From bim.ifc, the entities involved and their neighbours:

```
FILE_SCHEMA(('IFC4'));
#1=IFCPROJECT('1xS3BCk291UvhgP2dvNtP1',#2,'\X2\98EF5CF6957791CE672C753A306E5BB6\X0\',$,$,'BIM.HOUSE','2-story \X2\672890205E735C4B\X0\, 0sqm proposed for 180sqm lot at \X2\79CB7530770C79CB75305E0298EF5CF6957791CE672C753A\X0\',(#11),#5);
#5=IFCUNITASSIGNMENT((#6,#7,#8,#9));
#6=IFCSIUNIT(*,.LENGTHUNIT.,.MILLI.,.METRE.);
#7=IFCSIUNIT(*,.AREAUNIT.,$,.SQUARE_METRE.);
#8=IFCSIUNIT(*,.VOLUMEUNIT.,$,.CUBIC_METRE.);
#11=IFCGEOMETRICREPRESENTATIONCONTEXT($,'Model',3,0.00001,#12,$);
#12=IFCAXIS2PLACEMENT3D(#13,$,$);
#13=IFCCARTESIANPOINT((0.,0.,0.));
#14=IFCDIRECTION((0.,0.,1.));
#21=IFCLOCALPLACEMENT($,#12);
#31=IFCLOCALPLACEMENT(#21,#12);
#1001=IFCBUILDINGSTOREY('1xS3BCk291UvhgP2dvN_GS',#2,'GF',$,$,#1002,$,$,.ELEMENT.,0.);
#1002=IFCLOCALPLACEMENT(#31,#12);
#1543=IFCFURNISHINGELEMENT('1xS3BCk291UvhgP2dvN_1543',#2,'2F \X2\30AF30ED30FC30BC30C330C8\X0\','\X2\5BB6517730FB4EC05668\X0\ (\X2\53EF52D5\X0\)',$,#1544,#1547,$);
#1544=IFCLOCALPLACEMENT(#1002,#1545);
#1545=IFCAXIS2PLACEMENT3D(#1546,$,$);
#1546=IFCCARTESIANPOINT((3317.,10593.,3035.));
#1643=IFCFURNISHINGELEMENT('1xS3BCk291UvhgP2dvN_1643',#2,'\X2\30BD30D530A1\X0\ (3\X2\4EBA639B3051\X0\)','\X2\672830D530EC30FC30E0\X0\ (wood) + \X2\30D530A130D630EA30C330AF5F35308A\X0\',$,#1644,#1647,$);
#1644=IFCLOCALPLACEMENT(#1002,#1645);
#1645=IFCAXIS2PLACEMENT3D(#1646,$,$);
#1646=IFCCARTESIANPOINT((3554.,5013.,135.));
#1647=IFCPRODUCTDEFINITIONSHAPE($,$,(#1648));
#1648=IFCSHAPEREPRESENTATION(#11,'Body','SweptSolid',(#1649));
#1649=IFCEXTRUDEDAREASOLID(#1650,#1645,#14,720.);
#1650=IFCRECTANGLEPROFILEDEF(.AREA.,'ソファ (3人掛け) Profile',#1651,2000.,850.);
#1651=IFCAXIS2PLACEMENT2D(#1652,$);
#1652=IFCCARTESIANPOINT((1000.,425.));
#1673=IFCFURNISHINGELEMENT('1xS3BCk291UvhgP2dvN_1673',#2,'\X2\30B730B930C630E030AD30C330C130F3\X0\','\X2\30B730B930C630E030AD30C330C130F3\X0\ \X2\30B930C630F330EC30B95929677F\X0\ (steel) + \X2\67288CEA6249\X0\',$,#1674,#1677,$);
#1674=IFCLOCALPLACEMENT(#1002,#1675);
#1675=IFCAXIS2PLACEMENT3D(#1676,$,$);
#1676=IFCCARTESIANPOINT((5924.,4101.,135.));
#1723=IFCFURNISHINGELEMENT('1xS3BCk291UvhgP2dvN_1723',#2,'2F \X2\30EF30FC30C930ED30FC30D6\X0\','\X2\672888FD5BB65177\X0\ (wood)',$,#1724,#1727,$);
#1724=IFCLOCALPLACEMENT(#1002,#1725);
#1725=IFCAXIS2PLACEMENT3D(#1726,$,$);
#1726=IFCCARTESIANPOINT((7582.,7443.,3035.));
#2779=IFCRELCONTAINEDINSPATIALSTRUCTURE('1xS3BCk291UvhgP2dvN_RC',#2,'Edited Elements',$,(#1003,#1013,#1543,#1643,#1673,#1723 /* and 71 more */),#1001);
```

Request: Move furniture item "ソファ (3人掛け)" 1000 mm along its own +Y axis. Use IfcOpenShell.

```python
import ifcopenshell
import ifcopenshell.api.geometry
import ifcopenshell.util.placement
import ifcopenshell.util.unit

model = ifcopenshell.open("bim.ifc")
unit_scale = ifcopenshell.util.unit.calculate_unit_scale(model)

item = model.by_id(1643)
matrix = ifcopenshell.util.placement.get_local_placement(item.ObjectPlacement)
matrix[:3, 3] += matrix[:3, 1] * 1 / unit_scale
ifcopenshell.api.geometry.edit_object_placement(model, product=item, matrix=matrix, is_si=False)

print(ifcopenshell.util.placement.get_local_placement(item.ObjectPlacement).round(3) + 0.0)

model.write("bim_edited.ifc")
```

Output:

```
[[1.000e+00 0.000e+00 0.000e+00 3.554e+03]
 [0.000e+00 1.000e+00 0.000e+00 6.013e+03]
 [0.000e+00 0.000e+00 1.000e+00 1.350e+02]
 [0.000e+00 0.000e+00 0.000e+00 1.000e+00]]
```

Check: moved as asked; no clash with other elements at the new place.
